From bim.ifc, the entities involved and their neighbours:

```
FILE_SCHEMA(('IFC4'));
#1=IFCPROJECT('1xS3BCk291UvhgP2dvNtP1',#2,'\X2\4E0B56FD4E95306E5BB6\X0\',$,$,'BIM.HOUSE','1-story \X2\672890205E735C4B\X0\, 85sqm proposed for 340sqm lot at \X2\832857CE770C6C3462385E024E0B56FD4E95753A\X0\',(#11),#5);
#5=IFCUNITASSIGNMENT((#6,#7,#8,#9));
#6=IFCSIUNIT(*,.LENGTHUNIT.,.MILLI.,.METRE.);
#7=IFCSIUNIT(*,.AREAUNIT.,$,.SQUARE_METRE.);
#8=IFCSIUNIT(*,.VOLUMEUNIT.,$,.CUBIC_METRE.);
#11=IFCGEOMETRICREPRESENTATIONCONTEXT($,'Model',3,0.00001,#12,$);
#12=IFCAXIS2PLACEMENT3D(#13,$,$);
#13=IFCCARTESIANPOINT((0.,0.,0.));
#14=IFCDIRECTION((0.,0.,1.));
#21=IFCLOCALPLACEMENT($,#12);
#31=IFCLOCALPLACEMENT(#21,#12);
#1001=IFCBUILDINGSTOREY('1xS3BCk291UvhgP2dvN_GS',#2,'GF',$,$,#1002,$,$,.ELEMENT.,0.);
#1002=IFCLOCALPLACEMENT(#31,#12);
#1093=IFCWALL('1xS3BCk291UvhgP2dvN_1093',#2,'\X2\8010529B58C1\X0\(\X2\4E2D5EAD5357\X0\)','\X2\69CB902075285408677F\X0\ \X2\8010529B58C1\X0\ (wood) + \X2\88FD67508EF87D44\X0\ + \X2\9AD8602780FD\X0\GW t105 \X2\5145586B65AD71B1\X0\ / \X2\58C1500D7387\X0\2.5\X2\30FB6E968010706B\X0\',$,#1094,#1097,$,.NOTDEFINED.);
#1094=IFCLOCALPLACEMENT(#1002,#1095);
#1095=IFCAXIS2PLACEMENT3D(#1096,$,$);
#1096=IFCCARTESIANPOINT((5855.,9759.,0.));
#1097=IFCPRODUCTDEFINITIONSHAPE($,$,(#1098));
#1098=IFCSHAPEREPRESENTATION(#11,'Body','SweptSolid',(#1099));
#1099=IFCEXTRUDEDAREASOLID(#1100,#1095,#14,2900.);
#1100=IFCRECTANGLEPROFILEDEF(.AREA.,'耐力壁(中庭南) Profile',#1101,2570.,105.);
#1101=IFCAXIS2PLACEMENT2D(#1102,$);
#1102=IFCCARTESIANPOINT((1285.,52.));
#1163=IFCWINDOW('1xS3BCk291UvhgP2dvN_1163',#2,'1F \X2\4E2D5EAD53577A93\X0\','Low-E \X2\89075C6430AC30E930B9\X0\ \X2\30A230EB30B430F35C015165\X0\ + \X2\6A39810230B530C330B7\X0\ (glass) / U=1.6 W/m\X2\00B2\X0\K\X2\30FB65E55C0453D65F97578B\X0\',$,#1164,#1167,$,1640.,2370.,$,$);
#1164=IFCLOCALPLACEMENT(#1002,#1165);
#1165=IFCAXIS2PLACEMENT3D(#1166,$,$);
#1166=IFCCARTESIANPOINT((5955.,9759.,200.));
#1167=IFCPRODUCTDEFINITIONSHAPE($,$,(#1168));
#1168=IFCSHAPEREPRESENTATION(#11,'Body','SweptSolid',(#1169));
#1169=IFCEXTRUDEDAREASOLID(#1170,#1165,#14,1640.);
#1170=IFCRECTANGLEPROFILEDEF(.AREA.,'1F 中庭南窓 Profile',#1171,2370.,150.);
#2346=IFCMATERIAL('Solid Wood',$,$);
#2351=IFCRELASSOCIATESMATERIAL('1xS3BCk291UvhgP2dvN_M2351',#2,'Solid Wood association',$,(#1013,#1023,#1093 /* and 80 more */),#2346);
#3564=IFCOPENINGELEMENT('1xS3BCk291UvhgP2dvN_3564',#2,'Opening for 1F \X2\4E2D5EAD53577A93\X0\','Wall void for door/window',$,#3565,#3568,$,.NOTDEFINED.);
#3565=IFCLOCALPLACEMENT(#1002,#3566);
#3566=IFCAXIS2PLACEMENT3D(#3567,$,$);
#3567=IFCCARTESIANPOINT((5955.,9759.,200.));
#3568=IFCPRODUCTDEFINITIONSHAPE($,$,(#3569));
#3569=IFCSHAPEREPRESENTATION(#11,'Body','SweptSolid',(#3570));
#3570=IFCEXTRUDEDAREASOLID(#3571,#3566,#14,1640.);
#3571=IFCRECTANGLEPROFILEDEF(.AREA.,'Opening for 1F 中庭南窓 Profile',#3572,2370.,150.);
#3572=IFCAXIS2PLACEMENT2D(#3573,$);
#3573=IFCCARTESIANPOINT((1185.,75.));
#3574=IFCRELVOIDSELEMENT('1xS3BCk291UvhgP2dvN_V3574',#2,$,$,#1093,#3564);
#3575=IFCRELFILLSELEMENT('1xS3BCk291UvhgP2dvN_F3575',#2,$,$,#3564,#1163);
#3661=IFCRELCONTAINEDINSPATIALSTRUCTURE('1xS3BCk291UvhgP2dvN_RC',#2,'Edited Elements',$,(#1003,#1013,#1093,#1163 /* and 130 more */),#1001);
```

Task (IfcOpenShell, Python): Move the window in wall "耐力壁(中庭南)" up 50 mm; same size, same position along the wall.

```python
import numpy as np
import ifcopenshell
import ifcopenshell.api.geometry
import ifcopenshell.util.placement
import ifcopenshell.util.unit

model = ifcopenshell.open("bim.ifc")
unit_scale = ifcopenshell.util.unit.calculate_unit_scale(model)

window = model.by_guid("1xS3BCk291UvhgP2dvN_1163")
opening = window.FillsVoids[0].RelatingOpeningElement
dz = 0.05 / unit_scale

shift = np.array([0.0, 0.0, dz])
# The window is not placed relative to its opening, so move both.
for product in (opening, window):
    matrix = ifcopenshell.util.placement.get_local_placement(product.ObjectPlacement)
    matrix[:3, 3] += shift
    ifcopenshell.api.geometry.edit_object_placement(model, product=product, matrix=matrix, is_si=False)

print(f"moved by {dz * unit_scale:+.3f} m")

model.write("bim_rev.ifc")
```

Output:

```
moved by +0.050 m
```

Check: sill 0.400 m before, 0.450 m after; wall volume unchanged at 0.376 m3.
